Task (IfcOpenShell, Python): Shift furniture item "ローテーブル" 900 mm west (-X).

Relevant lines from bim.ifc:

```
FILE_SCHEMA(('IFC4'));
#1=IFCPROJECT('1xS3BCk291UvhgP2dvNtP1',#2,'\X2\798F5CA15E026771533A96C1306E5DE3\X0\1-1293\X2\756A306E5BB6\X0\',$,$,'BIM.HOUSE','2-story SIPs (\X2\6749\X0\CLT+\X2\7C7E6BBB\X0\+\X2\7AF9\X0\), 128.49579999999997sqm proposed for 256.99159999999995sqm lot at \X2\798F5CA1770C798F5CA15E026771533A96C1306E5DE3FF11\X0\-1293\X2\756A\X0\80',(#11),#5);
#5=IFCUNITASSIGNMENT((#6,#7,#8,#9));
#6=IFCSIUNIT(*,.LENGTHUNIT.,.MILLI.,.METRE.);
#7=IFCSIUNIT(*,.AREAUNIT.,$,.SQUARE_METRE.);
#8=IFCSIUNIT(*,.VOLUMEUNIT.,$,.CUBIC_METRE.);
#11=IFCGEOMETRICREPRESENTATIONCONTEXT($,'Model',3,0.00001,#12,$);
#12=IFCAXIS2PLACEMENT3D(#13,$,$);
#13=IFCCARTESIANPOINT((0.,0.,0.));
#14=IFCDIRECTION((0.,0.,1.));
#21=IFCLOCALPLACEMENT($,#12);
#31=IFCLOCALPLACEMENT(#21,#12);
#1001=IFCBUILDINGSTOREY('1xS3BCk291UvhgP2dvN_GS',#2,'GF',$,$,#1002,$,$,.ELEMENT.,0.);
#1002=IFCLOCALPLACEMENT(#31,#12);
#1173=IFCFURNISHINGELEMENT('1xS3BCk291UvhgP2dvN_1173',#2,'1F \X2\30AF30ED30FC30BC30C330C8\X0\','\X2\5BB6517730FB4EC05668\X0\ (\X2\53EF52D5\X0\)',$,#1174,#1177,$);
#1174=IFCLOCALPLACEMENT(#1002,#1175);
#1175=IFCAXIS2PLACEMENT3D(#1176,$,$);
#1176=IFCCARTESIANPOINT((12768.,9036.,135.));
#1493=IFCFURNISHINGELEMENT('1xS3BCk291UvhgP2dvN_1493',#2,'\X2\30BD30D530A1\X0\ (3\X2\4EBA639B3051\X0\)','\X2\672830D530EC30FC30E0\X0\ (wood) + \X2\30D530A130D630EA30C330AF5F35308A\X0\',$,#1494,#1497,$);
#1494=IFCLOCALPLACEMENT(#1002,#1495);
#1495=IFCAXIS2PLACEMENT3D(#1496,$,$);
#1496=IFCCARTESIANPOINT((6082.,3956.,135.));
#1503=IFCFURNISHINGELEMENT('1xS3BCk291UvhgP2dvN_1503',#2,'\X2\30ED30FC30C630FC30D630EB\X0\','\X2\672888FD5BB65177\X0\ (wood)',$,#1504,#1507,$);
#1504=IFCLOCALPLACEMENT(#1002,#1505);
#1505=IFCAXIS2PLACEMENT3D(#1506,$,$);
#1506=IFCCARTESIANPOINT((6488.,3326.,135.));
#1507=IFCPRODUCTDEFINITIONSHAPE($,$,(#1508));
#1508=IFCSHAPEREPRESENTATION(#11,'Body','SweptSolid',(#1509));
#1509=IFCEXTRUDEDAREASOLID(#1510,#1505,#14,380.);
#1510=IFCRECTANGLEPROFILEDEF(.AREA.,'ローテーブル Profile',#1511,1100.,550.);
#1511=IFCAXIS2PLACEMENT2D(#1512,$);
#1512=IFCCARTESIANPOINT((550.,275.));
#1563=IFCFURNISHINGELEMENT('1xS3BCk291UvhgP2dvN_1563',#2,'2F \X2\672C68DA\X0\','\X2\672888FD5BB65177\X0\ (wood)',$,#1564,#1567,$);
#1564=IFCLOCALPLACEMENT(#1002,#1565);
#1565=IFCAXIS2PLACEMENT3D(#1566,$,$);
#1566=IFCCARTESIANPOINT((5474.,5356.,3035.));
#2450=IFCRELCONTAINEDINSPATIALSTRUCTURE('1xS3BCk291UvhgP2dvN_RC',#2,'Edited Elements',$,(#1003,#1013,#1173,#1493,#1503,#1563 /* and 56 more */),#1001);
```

```python
import ifcopenshell
import ifcopenshell.api.geometry
import ifcopenshell.util.placement
import ifcopenshell.util.unit

model = ifcopenshell.open("bim.ifc")
unit_scale = ifcopenshell.util.unit.calculate_unit_scale(model)

item = model.by_id(1503)
matrix = ifcopenshell.util.placement.get_local_placement(item.ObjectPlacement)
matrix[0, 3] -= 0.9 / unit_scale
ifcopenshell.api.geometry.edit_object_placement(model, product=item, matrix=matrix, is_si=False)

print(ifcopenshell.util.placement.get_local_placement(item.ObjectPlacement).round(3) + 0.0)

model.write("bim-out.ifc")
```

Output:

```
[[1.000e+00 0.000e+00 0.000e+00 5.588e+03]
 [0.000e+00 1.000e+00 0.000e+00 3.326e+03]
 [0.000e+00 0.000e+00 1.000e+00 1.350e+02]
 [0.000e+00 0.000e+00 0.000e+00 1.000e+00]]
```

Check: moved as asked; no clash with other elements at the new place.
